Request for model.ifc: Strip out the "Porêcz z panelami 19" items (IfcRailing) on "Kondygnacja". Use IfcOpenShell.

First a look at what the model holds.

```python
import ifcopenshell
import ifcopenshell.util.element

model = ifcopenshell.open("model.ifc")
print(model.schema)
storey = next(s for s in model.by_type("IfcBuildingStorey") if s.Name == "Kondygnacja")
railings = [e for e in ifcopenshell.util.element.get_decomposition(storey) if e.is_a("IfcRailing")]
seen = {}
for e in railings:
    element_type = ifcopenshell.util.element.get_type(e)
    name = element_type.Name if element_type not in (None, e) else None
    seen[name] = seen.get(name, 0) + 1
for name, count in sorted(seen.items(), key=str):
    print(count, "x", name)
```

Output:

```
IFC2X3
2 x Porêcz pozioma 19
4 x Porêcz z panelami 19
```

```python
import ifcopenshell
import ifcopenshell.api.root
import ifcopenshell.util.element

model = ifcopenshell.open("model.ifc")

storey = next(s for s in model.by_type("IfcBuildingStorey") if s.Name == "Kondygnacja")
railings = [e for e in ifcopenshell.util.element.get_decomposition(storey) if e.is_a("IfcRailing")]
targets = [e for e in railings if (t := ifcopenshell.util.element.get_type(e)) not in (None, e) and t.Name == "Porêcz z panelami 19"]

for e in targets:
    ifcopenshell.api.root.remove_product(model, product=e)
print(len(targets), "removed")

model.write("model-out.ifc")
```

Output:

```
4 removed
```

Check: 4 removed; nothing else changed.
